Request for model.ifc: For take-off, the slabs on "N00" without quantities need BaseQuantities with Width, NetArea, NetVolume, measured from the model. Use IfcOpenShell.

First a look at what the model holds.

```python
import ifcopenshell
import ifcopenshell.util.element
import ifcopenshell.util.unit

model = ifcopenshell.open("model.ifc")
print(model.schema)
for unit_type in ("LENGTHUNIT", "AREAUNIT", "VOLUMEUNIT"):
    print(unit_type, ifcopenshell.util.unit.calculate_unit_scale(model, unit_type))
storey = next(s for s in model.by_type("IfcBuildingStorey") if s.Name == "N00")
slabs = [e for e in ifcopenshell.util.element.get_decomposition(storey) if e.is_a("IfcSlab")]
for e in sorted(slabs, key=lambda e: e.id()):
    print(e.id(), e.is_a(), e.Name, list(ifcopenshell.util.element.get_psets(e, qtos_only=True)), sep=" | ")
```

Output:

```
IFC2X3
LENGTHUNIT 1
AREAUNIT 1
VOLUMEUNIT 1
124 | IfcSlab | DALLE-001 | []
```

```python
import ifcopenshell
import ifcopenshell.api.pset
import ifcopenshell.geom
import ifcopenshell.util.element
import ifcopenshell.util.shape
import ifcopenshell.util.unit

model = ifcopenshell.open("model.ifc")
unit_scale = ifcopenshell.util.unit.calculate_unit_scale(model)
area_scale = ifcopenshell.util.unit.calculate_unit_scale(model, "AREAUNIT")
volume_scale = ifcopenshell.util.unit.calculate_unit_scale(model, "VOLUMEUNIT")
settings = ifcopenshell.geom.settings()

storey = next(s for s in model.by_type("IfcBuildingStorey") if s.Name == "N00")
slabs = [e for e in ifcopenshell.util.element.get_decomposition(storey) if e.is_a("IfcSlab")]

for e in sorted(slabs, key=lambda e: e.id()):
    if ifcopenshell.util.element.get_psets(e, qtos_only=True, should_inherit=False):
        continue
    # Geometry comes back in metres, in the element's own axes.
    shape = ifcopenshell.geom.create_shape(settings, e)
    values = {
        "Width": ifcopenshell.util.shape.get_z(shape.geometry) / unit_scale,
        "NetArea": ifcopenshell.util.shape.get_footprint_area(shape.geometry) / area_scale,
        "NetVolume": ifcopenshell.util.shape.get_volume(shape.geometry) / volume_scale,
    }
    qto = ifcopenshell.api.pset.add_qto(model, product=e, name="BaseQuantities")
    ifcopenshell.api.pset.edit_qto(model, qto=qto, properties=values)
    print(e.id(), {k: round(v, 3) for k, v in values.items()})

model.write("model_edited.ifc")
```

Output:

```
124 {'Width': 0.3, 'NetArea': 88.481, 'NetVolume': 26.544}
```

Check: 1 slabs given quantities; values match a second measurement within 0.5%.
